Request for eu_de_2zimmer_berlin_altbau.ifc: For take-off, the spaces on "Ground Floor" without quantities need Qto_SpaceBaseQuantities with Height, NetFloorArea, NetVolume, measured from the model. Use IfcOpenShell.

First a look at what the model holds.

```python
import ifcopenshell
import ifcopenshell.util.element
import ifcopenshell.util.unit

model = ifcopenshell.open("eu_de_2zimmer_berlin_altbau.ifc")
print(model.schema)
for unit_type in ("LENGTHUNIT", "AREAUNIT", "VOLUMEUNIT"):
    print(unit_type, ifcopenshell.util.unit.calculate_unit_scale(model, unit_type))
storey = next(s for s in model.by_type("IfcBuildingStorey") if s.Name == "Ground Floor")
spaces = [e for e in ifcopenshell.util.element.get_decomposition(storey) if e.is_a("IfcSpace")]
for e in sorted(spaces, key=lambda e: e.id()):
    print(e.id(), e.is_a(), e.Name, list(ifcopenshell.util.element.get_psets(e, qtos_only=True)), sep=" | ")
```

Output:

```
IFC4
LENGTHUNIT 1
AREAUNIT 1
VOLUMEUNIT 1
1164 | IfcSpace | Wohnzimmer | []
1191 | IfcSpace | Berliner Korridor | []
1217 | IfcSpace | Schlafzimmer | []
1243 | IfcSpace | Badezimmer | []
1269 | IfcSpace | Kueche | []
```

```python
import ifcopenshell
import ifcopenshell.api.pset
import ifcopenshell.geom
import ifcopenshell.util.element
import ifcopenshell.util.shape
import ifcopenshell.util.unit

model = ifcopenshell.open("eu_de_2zimmer_berlin_altbau.ifc")
unit_scale = ifcopenshell.util.unit.calculate_unit_scale(model)
area_scale = ifcopenshell.util.unit.calculate_unit_scale(model, "AREAUNIT")
volume_scale = ifcopenshell.util.unit.calculate_unit_scale(model, "VOLUMEUNIT")
settings = ifcopenshell.geom.settings()

storey = next(s for s in model.by_type("IfcBuildingStorey") if s.Name == "Ground Floor")
spaces = [e for e in ifcopenshell.util.element.get_decomposition(storey) if e.is_a("IfcSpace")]

for e in sorted(spaces, key=lambda e: e.id()):
    if ifcopenshell.util.element.get_psets(e, qtos_only=True, should_inherit=False):
        continue
    # Geometry comes back in metres, in the element's own axes.
    shape = ifcopenshell.geom.create_shape(settings, e)
    values = {
        "Height": ifcopenshell.util.shape.get_z(shape.geometry) / unit_scale,
        "NetFloorArea": ifcopenshell.util.shape.get_footprint_area(shape.geometry) / area_scale,
        "NetVolume": ifcopenshell.util.shape.get_volume(shape.geometry) / volume_scale,
    }
    qto = ifcopenshell.api.pset.add_qto(model, product=e, name="Qto_SpaceBaseQuantities")
    ifcopenshell.api.pset.edit_qto(model, qto=qto, properties=values)
    print(e.id(), {k: round(v, 3) for k, v in values.items()})

model.write("eu_de_2zimmer_berlin_altbau_updated.ifc")
```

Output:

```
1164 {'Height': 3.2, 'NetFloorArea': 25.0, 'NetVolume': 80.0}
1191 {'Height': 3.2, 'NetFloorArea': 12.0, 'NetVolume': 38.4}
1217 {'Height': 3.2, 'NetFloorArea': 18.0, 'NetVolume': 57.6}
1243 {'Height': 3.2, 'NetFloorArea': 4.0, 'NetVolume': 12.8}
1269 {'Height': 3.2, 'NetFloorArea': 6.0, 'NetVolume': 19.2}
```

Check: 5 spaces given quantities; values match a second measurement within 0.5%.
